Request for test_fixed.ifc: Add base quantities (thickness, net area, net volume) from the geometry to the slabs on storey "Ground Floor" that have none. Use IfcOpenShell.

First a look at what the model holds.

```python
import ifcopenshell
import ifcopenshell.util.element
import ifcopenshell.util.unit

model = ifcopenshell.open("test_fixed.ifc")
print(model.schema)
for unit_type in ("LENGTHUNIT", "AREAUNIT", "VOLUMEUNIT"):
    print(unit_type, ifcopenshell.util.unit.calculate_unit_scale(model, unit_type))
storey = next(s for s in model.by_type("IfcBuildingStorey") if s.Name == "Ground Floor")
slabs = [e for e in ifcopenshell.util.element.get_decomposition(storey) if e.is_a("IfcSlab")]
for e in sorted(slabs, key=lambda e: e.id()):
    print(e.id(), e.is_a(), e.Name, list(ifcopenshell.util.element.get_psets(e, qtos_only=True)), sep=" | ")
```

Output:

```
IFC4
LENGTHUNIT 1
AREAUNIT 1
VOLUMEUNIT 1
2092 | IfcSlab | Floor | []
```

```python
import ifcopenshell
import ifcopenshell.api.pset
import ifcopenshell.geom
import ifcopenshell.util.element
import ifcopenshell.util.shape
import ifcopenshell.util.unit

model = ifcopenshell.open("test_fixed.ifc")
unit_scale = ifcopenshell.util.unit.calculate_unit_scale(model)
area_scale = ifcopenshell.util.unit.calculate_unit_scale(model, "AREAUNIT")
volume_scale = ifcopenshell.util.unit.calculate_unit_scale(model, "VOLUMEUNIT")
settings = ifcopenshell.geom.settings()

storey = next(s for s in model.by_type("IfcBuildingStorey") if s.Name == "Ground Floor")
slabs = [e for e in ifcopenshell.util.element.get_decomposition(storey) if e.is_a("IfcSlab")]

for e in sorted(slabs, key=lambda e: e.id()):
    if ifcopenshell.util.element.get_psets(e, qtos_only=True, should_inherit=False):
        continue
    # Geometry comes back in metres, in the element's own axes.
    shape = ifcopenshell.geom.create_shape(settings, e)
    values = {
        "Width": ifcopenshell.util.shape.get_z(shape.geometry) / unit_scale,
        "NetArea": ifcopenshell.util.shape.get_footprint_area(shape.geometry) / area_scale,
        "NetVolume": ifcopenshell.util.shape.get_volume(shape.geometry) / volume_scale,
    }
    qto = ifcopenshell.api.pset.add_qto(model, product=e, name="Qto_SlabBaseQuantities")
    ifcopenshell.api.pset.edit_qto(model, qto=qto, properties=values)
    print(e.id(), {k: round(v, 3) for k, v in values.items()})

model.write("test_fixed_v2.ifc")
```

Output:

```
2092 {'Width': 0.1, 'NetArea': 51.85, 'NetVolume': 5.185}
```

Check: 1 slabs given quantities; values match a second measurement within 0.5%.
